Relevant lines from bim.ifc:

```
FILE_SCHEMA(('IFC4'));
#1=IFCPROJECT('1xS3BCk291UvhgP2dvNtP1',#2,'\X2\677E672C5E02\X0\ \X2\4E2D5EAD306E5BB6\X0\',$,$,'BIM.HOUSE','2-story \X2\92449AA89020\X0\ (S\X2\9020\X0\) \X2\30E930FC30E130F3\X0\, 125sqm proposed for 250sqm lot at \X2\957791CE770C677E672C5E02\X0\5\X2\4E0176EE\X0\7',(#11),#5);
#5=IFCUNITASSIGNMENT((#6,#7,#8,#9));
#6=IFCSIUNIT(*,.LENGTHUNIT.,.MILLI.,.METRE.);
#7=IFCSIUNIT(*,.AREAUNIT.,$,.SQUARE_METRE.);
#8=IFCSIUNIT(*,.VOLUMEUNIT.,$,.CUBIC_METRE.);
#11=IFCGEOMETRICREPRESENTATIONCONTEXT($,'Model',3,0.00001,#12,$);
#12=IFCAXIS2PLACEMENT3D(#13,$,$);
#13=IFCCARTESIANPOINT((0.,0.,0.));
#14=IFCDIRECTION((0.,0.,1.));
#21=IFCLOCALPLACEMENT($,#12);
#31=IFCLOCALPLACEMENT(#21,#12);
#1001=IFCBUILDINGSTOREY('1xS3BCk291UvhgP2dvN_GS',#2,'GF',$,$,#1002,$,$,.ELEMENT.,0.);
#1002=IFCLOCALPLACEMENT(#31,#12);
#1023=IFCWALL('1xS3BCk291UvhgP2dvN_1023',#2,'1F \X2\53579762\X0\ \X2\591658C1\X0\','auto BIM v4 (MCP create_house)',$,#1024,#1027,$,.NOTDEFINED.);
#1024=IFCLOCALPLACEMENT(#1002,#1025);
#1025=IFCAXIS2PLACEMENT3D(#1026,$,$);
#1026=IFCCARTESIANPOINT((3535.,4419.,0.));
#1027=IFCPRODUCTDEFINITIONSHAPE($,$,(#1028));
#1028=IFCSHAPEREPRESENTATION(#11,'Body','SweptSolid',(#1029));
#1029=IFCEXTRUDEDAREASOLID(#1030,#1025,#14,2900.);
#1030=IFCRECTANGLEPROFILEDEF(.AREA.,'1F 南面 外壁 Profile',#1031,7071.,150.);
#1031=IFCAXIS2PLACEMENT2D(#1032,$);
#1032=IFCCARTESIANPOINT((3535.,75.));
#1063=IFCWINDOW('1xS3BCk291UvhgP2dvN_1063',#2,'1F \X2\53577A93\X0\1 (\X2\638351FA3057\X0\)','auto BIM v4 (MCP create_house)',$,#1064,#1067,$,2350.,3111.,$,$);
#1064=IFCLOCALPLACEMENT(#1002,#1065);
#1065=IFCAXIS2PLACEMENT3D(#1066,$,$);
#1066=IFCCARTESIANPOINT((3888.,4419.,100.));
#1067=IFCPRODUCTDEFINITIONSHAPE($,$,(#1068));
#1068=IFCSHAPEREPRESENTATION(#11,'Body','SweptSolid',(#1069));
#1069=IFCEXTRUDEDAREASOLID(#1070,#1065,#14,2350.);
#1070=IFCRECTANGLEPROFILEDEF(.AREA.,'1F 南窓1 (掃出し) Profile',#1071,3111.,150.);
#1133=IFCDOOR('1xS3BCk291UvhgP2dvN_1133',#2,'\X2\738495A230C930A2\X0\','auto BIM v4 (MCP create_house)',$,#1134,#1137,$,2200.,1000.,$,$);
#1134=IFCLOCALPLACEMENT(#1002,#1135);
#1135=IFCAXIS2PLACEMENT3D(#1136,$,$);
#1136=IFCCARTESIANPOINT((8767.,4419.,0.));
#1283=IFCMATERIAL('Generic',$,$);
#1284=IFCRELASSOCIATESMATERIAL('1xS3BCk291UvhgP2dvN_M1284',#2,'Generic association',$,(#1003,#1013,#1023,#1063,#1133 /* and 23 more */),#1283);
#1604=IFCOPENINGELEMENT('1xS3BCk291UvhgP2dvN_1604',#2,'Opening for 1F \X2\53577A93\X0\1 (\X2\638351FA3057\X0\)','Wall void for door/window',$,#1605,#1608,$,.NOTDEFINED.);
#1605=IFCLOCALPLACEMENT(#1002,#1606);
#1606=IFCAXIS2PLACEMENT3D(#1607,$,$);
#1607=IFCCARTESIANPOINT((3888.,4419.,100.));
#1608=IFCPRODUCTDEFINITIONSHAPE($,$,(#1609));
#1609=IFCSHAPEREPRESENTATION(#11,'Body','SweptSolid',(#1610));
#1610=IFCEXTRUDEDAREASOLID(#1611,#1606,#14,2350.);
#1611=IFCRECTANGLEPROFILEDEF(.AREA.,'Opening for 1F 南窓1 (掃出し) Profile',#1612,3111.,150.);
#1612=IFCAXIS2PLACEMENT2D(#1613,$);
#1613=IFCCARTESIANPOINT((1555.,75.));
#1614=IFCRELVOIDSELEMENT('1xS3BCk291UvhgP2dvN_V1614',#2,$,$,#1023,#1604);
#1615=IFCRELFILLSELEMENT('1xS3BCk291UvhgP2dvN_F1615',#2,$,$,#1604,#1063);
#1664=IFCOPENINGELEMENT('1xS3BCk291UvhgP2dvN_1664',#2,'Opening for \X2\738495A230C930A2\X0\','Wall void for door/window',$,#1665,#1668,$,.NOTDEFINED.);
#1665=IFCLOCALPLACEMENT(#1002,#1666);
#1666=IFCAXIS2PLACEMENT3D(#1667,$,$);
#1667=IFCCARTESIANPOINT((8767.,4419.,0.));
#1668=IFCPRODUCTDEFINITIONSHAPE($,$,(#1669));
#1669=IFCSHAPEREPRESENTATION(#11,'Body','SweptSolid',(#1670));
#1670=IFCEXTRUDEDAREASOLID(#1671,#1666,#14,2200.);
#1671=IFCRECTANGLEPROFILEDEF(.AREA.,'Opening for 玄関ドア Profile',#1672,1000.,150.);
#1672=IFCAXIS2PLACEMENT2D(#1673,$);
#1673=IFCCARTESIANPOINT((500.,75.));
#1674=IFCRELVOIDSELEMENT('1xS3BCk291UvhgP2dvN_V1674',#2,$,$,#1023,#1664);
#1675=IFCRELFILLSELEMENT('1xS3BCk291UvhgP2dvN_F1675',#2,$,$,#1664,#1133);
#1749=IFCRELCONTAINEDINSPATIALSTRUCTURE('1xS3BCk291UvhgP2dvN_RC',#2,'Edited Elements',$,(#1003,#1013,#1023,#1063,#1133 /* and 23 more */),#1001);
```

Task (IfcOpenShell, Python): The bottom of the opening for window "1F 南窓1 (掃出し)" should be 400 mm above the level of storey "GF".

```python
import numpy as np
import ifcopenshell
import ifcopenshell.api.geometry
import ifcopenshell.geom
import ifcopenshell.util.element
import ifcopenshell.util.placement
import ifcopenshell.util.shape
import ifcopenshell.util.unit

model = ifcopenshell.open("bim.ifc")
unit_scale = ifcopenshell.util.unit.calculate_unit_scale(model)

window = model.by_guid("1xS3BCk291UvhgP2dvN_1063")
opening = window.FillsVoids[0].RelatingOpeningElement
storey = ifcopenshell.util.element.get_container(window, ifc_class="IfcBuildingStorey")
level = ifcopenshell.util.placement.get_local_placement(storey.ObjectPlacement)[2, 3]

# The opening's origin need not be at the sill, so measure its lowest point.
shape = ifcopenshell.geom.create_shape(ifcopenshell.geom.settings(), opening)
bottom = ifcopenshell.util.shape.get_shape_bottom_elevation(shape, shape.geometry) / unit_scale
dz = level + 0.4 / unit_scale - bottom

shift = np.array([0.0, 0.0, dz])
# The window is not placed relative to its opening, so move both.
for product in (opening, window):
    matrix = ifcopenshell.util.placement.get_local_placement(product.ObjectPlacement)
    matrix[:3, 3] += shift
    ifcopenshell.api.geometry.edit_object_placement(model, product=product, matrix=matrix, is_si=False)

print(f"moved by {dz * unit_scale:+.3f} m")

model.write("bim_updated.ifc")
```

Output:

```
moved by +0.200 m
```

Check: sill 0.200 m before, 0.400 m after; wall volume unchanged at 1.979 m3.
